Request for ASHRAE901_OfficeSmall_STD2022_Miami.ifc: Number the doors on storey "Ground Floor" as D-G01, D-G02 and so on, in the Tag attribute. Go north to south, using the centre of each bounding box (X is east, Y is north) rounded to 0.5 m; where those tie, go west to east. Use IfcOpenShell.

First a look at what the model holds.

```python
import ifcopenshell
import ifcopenshell.util.element
import ifcopenshell.util.placement

model = ifcopenshell.open("ASHRAE901_OfficeSmall_STD2022_Miami.ifc")
print(model.schema)
storey = next(s for s in model.by_type("IfcBuildingStorey") if s.Name == "Ground Floor")
doors = [e for e in ifcopenshell.util.element.get_decomposition(storey) if e.is_a("IfcDoor")]
for e in sorted(doors, key=lambda e: e.id()):
    origin = ifcopenshell.util.placement.get_local_placement(e.ObjectPlacement)[:3, 3]
    print(e.id(), e.Tag, e.Name, origin.round(2) + 0.0, sep=" | ")
```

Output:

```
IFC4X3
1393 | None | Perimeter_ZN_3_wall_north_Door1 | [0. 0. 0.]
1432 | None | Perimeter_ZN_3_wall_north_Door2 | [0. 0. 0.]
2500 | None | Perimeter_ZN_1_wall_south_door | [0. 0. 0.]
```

```python
import ifcopenshell
import ifcopenshell.geom
import ifcopenshell.util.element
import ifcopenshell.util.shape

model = ifcopenshell.open("ASHRAE901_OfficeSmall_STD2022_Miami.ifc")
settings = ifcopenshell.geom.settings()
settings.set("use-world-coords", True)


def centre(element):
    shape = ifcopenshell.geom.create_shape(settings, element)
    return ifcopenshell.util.shape.get_bbox_centroid(shape.geometry)


storey = next(s for s in model.by_type("IfcBuildingStorey") if s.Name == "Ground Floor")
doors = [e for e in ifcopenshell.util.element.get_decomposition(storey) if e.is_a("IfcDoor")]

# Insertion points can sit at a corner or the storey origin, so sort by the geometry (in metres).
centres = {e: centre(e) for e in doors}
doors.sort(key=lambda e: (-round(centres[e][1] / 0.5), centres[e][0]))

for i, e in enumerate(doors, start=1):
    number = f"D-G{i:02d}"
    e.Tag = number
    print(e.id(), number)

model.write("ASHRAE901_OfficeSmall_STD2022_Miami_updated.ifc")
```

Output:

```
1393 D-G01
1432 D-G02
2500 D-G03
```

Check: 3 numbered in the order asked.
